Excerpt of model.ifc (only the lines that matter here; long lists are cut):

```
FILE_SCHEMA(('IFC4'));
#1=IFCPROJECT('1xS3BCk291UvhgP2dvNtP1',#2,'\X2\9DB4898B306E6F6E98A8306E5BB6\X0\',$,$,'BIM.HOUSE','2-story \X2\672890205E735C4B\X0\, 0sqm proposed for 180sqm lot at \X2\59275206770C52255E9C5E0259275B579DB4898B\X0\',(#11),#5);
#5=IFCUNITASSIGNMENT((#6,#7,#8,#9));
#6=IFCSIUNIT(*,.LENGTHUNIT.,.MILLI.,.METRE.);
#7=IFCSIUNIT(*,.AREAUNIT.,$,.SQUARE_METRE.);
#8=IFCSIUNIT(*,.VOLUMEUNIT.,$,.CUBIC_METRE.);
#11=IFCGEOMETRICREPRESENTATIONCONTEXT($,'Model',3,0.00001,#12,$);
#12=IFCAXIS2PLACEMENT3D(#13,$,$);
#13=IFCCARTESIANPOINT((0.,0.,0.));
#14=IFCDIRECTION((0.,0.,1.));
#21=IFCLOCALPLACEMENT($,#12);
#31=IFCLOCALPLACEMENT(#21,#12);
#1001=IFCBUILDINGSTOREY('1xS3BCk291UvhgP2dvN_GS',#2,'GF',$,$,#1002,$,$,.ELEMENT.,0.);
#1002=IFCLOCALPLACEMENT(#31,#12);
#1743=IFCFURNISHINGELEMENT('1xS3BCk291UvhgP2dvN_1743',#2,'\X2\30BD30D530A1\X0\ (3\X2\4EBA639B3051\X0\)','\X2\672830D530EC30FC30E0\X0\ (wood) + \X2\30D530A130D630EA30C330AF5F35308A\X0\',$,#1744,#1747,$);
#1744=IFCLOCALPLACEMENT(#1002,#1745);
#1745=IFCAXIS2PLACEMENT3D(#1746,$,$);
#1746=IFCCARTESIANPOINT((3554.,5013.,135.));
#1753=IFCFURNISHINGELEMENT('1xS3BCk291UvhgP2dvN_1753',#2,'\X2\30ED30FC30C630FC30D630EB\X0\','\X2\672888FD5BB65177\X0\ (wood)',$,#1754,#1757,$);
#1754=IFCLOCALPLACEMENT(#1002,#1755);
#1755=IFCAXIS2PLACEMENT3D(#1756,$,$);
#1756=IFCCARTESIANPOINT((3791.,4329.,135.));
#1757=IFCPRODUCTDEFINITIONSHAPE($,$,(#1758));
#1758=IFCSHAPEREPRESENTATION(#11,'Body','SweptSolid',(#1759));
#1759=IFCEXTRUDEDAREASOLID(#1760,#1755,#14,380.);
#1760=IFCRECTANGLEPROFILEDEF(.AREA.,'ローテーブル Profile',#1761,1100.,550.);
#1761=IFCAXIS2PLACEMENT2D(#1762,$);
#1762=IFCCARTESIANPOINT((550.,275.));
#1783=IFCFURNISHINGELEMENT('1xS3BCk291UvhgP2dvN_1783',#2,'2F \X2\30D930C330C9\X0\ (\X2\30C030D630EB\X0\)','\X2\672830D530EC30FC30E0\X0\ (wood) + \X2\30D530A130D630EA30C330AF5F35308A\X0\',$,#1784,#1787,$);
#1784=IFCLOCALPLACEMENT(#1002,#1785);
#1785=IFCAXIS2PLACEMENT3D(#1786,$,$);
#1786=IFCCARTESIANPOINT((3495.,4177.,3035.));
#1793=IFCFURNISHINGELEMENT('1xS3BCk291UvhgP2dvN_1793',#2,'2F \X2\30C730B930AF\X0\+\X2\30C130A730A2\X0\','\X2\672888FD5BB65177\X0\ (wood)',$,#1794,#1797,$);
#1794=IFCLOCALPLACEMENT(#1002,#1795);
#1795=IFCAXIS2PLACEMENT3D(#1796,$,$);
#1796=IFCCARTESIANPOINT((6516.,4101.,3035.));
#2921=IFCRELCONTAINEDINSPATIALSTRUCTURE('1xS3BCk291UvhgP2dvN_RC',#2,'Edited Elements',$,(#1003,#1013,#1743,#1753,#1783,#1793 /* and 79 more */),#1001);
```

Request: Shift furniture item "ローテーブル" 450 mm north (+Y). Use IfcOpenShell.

```python
import ifcopenshell
import ifcopenshell.api.geometry
import ifcopenshell.util.placement

model = ifcopenshell.open("model.ifc")

item = model.by_guid("1xS3BCk291UvhgP2dvN_1753")
matrix = ifcopenshell.util.placement.get_local_placement(item.ObjectPlacement)
matrix[1, 3] += 450.0
ifcopenshell.api.geometry.edit_object_placement(model, product=item, matrix=matrix, is_si=False)

print(ifcopenshell.util.placement.get_local_placement(item.ObjectPlacement).round(3) + 0.0)

model.write("model_updated.ifc")
```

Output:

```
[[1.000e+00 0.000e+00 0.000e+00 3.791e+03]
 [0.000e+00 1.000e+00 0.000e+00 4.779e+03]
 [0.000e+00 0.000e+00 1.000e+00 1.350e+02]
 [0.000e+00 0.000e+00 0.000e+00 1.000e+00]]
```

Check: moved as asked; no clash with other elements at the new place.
